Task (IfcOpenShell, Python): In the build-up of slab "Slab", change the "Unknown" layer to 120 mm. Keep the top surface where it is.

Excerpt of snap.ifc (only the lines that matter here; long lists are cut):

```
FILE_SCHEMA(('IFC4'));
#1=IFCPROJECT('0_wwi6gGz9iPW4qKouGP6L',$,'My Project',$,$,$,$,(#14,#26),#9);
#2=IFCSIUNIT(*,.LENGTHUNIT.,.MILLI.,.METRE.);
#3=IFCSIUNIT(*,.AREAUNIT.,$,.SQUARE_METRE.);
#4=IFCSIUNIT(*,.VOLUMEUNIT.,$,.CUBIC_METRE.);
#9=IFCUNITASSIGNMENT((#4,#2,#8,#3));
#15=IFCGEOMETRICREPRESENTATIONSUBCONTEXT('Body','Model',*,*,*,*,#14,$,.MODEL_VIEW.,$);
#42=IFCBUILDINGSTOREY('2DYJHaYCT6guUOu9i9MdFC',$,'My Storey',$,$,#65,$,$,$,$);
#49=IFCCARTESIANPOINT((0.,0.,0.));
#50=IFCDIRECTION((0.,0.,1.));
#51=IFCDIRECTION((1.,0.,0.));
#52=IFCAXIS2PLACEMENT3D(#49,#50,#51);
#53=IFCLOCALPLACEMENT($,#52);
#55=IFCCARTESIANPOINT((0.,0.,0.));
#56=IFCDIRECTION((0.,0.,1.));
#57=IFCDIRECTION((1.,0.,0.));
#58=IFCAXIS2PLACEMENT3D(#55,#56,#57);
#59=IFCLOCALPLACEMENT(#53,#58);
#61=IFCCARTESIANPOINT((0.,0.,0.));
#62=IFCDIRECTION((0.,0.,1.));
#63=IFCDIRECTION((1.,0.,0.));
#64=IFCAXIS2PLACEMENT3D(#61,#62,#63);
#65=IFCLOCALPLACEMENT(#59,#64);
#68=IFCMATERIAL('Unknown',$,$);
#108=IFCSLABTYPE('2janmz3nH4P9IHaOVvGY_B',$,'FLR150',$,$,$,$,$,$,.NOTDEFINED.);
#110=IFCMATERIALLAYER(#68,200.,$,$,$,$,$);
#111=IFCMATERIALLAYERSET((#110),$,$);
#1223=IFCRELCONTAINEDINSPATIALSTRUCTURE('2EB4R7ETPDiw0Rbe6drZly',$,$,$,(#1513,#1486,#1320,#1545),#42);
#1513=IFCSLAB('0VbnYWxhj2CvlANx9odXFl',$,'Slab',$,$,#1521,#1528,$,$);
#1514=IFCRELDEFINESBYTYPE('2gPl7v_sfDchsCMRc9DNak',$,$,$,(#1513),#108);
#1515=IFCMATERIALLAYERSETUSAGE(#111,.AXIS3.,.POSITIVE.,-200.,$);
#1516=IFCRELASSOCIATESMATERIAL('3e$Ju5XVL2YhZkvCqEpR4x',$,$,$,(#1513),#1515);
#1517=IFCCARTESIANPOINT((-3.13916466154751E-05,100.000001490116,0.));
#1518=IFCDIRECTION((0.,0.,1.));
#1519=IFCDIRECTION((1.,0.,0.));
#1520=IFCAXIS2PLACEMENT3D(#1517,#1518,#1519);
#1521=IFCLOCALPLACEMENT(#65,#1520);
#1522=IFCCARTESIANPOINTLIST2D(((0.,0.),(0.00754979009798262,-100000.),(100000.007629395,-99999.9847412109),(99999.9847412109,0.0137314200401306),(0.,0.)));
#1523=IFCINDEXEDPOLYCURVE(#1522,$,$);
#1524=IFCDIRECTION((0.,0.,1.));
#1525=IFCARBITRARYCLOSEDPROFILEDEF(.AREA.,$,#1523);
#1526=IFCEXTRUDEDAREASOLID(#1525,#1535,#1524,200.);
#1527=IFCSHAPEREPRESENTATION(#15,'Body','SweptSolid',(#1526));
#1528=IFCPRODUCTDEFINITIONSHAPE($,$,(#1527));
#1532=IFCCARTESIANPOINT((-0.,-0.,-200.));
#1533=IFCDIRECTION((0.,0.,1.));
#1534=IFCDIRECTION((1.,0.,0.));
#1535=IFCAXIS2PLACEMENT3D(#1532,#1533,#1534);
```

```python
import ifcopenshell
import ifcopenshell.util.element
import ifcopenshell.util.representation
import ifcopenshell.util.unit

model = ifcopenshell.open("snap.ifc")
unit_scale = ifcopenshell.util.unit.calculate_unit_scale(model)

layer_set = model.by_id(111)
layer = next(l for l in layer_set.MaterialLayers if l.Material and l.Material.Name == "Unknown")
change = 0.12 / unit_scale - layer.LayerThickness
layer.LayerThickness += change

# Geometry does not follow the layer set by itself.
slabs = [e for e in ifcopenshell.util.element.get_elements_by_material(model, layer_set) if e.is_a("IfcSlab")]
for slab in sorted(slabs, key=lambda e: e.id()):
    body = ifcopenshell.util.representation.get_representation(slab, "Model", "Body")
    solid = body.Items[0]
    old_depth = solid.Depth
    solid.Depth += change
    # Extruded upwards: lower the start of the extrusion so the top stays.
    x, y, z = solid.Position.Location.Coordinates
    solid.Position.Location = model.createIfcCartesianPoint((x, y, z - change))
    print(slab.id(), f"{old_depth:g} -> {solid.Depth:g}")

# The layers are counted up from the underside, which has moved.
for usage in {ifcopenshell.util.element.get_material(slab) for slab in slabs}:
    usage.OffsetFromReferenceLine -= change

model.write("snap-out.ifc")
```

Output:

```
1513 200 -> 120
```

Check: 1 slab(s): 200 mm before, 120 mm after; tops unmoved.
